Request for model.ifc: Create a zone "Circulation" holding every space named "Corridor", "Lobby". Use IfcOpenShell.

First a look at what the model holds.

```python
import ifcopenshell

model = ifcopenshell.open("model.ifc")
print(model.schema)
seen = {}
for space in model.by_type("IfcSpace"):
    seen[space.LongName] = seen.get(space.LongName, 0) + 1
for name, count in sorted(seen.items(), key=str):
    print(count, "x", name)
print("zones:", [z.Name for z in model.by_type("IfcZone")][:20])
```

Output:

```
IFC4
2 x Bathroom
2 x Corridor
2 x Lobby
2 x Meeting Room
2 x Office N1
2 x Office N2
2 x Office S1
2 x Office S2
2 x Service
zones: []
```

```python
import ifcopenshell
import ifcopenshell.api.group
import ifcopenshell.api.root

model = ifcopenshell.open("model.ifc")

names = {"Corridor", "Lobby"}
spaces = [s for s in model.by_type("IfcSpace") if s.LongName in names]

zone = ifcopenshell.api.root.create_entity(model, ifc_class="IfcZone", name="Circulation")
ifcopenshell.api.group.assign_group(model, products=spaces, group=zone)
print(len(spaces), "spaces in", zone.Name)

model.write("model_updated.ifc")
```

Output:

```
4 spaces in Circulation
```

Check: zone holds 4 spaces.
